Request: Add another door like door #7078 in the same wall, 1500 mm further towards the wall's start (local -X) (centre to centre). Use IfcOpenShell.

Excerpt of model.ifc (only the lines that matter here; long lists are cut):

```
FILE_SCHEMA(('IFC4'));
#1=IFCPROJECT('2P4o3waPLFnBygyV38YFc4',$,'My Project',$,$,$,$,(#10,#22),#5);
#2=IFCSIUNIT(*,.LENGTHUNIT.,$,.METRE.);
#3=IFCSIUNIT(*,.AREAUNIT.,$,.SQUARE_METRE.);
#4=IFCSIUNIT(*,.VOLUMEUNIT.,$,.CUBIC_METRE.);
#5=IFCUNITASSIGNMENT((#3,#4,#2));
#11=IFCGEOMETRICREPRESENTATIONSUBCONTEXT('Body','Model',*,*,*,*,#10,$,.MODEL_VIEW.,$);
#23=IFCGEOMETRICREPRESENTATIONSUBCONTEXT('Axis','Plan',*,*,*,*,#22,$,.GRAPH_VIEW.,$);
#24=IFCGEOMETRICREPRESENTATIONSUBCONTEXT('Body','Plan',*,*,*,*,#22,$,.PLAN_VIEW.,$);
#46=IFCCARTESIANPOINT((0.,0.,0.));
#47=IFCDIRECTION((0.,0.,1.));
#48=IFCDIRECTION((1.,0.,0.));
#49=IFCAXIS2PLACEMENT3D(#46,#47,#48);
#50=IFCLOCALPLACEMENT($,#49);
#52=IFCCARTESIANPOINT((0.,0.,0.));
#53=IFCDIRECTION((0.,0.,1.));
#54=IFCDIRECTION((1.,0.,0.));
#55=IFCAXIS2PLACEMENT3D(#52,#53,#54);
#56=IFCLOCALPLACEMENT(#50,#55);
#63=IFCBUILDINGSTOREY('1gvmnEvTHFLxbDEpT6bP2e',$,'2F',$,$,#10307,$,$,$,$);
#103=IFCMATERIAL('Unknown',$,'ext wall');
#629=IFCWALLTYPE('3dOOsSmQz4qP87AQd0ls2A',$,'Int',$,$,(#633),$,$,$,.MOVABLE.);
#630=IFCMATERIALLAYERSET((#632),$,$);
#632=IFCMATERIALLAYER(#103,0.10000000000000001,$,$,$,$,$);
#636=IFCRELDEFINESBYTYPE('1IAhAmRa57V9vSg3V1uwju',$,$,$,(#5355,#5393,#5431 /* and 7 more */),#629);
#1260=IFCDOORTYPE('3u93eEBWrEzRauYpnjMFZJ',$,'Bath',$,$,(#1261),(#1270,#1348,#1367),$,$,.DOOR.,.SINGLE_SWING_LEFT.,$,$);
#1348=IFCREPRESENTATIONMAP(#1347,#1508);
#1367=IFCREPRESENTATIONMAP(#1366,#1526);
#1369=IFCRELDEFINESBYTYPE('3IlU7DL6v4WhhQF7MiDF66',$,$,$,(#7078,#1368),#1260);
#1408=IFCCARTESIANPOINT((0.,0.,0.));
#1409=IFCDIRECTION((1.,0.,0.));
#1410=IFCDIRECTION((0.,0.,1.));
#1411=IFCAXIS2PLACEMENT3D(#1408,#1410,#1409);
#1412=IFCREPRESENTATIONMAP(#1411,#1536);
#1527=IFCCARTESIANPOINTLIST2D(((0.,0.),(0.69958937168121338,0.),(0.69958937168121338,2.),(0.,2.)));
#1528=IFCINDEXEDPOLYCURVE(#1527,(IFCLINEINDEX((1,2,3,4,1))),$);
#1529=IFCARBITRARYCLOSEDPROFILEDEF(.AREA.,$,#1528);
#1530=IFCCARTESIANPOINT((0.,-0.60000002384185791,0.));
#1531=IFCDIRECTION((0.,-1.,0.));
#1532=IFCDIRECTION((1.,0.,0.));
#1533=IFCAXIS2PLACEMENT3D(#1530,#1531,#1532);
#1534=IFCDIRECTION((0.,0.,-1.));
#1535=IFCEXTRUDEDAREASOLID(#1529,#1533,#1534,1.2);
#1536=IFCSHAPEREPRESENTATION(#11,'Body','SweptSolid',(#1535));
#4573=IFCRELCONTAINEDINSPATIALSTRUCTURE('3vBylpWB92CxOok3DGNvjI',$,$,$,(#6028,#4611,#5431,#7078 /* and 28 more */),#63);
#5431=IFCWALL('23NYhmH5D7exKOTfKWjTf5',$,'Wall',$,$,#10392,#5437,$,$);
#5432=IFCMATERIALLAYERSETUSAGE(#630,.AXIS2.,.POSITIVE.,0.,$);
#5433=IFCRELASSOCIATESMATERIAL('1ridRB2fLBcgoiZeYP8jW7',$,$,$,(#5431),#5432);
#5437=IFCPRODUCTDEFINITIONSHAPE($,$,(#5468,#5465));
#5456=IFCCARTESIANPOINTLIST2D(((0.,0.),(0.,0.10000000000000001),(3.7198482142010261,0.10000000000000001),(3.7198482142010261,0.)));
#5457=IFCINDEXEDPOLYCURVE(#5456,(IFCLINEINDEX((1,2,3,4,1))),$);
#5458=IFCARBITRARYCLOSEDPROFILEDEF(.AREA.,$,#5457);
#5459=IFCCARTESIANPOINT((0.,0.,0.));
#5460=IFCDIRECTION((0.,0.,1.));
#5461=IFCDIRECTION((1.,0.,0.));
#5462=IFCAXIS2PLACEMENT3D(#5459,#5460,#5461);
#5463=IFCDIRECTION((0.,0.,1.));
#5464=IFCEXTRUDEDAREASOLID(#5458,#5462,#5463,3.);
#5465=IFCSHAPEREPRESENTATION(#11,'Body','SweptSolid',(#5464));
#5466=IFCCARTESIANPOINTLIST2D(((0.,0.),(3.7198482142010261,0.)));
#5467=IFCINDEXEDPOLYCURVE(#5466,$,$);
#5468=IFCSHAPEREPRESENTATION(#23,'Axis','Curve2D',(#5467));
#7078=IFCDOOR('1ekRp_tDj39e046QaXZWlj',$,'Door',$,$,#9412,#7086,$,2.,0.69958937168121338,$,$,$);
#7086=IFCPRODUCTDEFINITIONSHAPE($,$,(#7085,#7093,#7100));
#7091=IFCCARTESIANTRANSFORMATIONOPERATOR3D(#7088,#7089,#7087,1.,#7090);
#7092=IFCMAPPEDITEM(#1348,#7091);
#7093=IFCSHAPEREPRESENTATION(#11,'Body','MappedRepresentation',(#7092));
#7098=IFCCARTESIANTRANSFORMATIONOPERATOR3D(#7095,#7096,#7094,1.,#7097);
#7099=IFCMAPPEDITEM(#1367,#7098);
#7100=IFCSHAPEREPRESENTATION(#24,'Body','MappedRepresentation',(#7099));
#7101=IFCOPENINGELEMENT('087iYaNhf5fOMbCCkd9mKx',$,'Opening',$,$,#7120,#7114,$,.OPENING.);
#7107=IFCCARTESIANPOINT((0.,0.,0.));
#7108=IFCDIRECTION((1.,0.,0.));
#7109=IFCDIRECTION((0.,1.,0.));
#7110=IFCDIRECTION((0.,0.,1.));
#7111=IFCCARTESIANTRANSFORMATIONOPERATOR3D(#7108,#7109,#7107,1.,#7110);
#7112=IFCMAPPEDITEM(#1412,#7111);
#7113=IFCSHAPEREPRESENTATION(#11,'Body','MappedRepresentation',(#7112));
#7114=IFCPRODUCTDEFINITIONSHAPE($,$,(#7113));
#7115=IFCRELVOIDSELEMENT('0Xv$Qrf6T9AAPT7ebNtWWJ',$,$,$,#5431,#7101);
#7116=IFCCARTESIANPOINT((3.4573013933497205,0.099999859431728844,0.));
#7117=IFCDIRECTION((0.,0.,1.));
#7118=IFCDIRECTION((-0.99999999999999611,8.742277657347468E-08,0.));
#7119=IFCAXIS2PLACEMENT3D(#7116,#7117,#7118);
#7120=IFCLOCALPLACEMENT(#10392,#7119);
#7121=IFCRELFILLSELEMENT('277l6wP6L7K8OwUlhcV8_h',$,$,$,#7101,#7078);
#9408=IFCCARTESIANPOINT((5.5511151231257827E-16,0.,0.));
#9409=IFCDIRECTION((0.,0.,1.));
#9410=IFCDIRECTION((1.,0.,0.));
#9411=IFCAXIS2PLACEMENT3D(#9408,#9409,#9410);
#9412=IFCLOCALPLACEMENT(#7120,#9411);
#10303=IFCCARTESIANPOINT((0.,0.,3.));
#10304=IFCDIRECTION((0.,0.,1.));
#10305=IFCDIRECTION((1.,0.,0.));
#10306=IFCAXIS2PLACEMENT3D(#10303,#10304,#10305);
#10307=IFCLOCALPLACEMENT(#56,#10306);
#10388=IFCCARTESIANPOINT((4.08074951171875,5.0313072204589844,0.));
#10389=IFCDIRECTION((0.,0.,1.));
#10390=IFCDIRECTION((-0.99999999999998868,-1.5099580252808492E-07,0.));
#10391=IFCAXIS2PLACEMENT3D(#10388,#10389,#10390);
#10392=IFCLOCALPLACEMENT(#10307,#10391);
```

```python
import ifcopenshell
import ifcopenshell.api.feature
import ifcopenshell.api.geometry
import ifcopenshell.api.root
import ifcopenshell.geom
import ifcopenshell.util.element
import ifcopenshell.util.placement
import ifcopenshell.util.shape
import ifcopenshell.util.unit

model = ifcopenshell.open("model.ifc")
unit_scale = ifcopenshell.util.unit.calculate_unit_scale(model)
settings = ifcopenshell.geom.settings()


def volume(element):
    """Net volume in cubic metres, openings subtracted."""
    shape = ifcopenshell.geom.create_shape(settings, element)
    return ifcopenshell.util.shape.get_volume(shape.geometry)


door = model.by_id(7078)
opening = door.FillsVoids[0].RelatingOpeningElement
wall = opening.VoidsElements[0].RelatingBuildingElement
before = volume(wall)
shift = ifcopenshell.util.placement.get_local_placement(wall.ObjectPlacement)[:3, 0] * -1.5 / unit_scale

# copy_class copies the void relationship, type, container and properties, but no geometry.
new_opening = ifcopenshell.api.root.copy_class(model, product=opening)
new_opening.Representation = ifcopenshell.util.element.copy_deep(
    model, opening.Representation, exclude=["IfcGeometricRepresentationContext", "IfcRepresentationMap"]
)
new_door = ifcopenshell.api.root.copy_class(model, product=door)
new_door.Representation = ifcopenshell.util.element.copy_deep(
    model, door.Representation, exclude=["IfcGeometricRepresentationContext", "IfcRepresentationMap"]
)
ifcopenshell.api.feature.add_filling(model, opening=new_opening, element=new_door)

for old, new in ((opening, new_opening), (door, new_door)):
    matrix = ifcopenshell.util.placement.get_local_placement(old.ObjectPlacement)
    matrix[:3, 3] += shift
    ifcopenshell.api.geometry.edit_object_placement(model, product=new, matrix=matrix, is_si=False)

after = volume(wall)

print(f"wall volume {before:.3f} -> {after:.3f} m3")

model.write("model_rev.ifc")
```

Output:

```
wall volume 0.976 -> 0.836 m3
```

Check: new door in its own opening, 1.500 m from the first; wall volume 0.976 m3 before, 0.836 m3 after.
